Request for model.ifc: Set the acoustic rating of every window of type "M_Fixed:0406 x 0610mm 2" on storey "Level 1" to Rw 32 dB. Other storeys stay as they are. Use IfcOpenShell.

First a look at what the model holds.

```python
import ifcopenshell
import ifcopenshell.util.element

model = ifcopenshell.open("model.ifc")
print(model.schema)
storey = next(s for s in model.by_type("IfcBuildingStorey") if s.Name == "Level 1")
windows = [e for e in ifcopenshell.util.element.get_decomposition(storey) if e.is_a("IfcWindow")]
seen = {}
for e in windows:
    element_type = ifcopenshell.util.element.get_type(e)
    key = (element_type.Name if element_type != e and element_type else None, ifcopenshell.util.element.get_pset(e, "Pset_WindowCommon", "AcousticRating"))
    seen[key] = seen.get(key, 0) + 1
for (name, value), count in sorted(seen.items(), key=str):
    print(count, "x", name, "|", value)
```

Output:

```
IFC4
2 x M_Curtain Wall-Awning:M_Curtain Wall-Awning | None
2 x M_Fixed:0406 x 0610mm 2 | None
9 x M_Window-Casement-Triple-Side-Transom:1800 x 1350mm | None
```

```python
import ifcopenshell
import ifcopenshell.api.pset
import ifcopenshell.util.element

model = ifcopenshell.open("model.ifc")

storey = next(s for s in model.by_type("IfcBuildingStorey") if s.Name == "Level 1")
windows = [e for e in ifcopenshell.util.element.get_decomposition(storey) if e.is_a("IfcWindow")]

count = 0
for e in windows:
    element_type = ifcopenshell.util.element.get_type(e)
    if element_type in (None, e) or element_type.Name != "M_Fixed:0406 x 0610mm 2":
        continue
    # add_pset returns the element's existing set when there is one.
    pset = ifcopenshell.api.pset.add_pset(model, product=e, name="Pset_WindowCommon")
    ifcopenshell.api.pset.edit_pset(model, pset=pset, properties={"AcousticRating": "Rw 32 dB"})
    count += 1

print(count, "windows updated")

model.write("model_edited.ifc")
```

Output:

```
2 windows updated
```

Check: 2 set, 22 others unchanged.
